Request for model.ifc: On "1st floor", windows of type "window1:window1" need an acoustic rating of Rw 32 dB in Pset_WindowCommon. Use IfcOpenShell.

First a look at what the model holds.

```python
import ifcopenshell
import ifcopenshell.util.element

model = ifcopenshell.open("model.ifc")
print(model.schema)
storey = next(s for s in model.by_type("IfcBuildingStorey") if s.Name == "1st floor")
windows = [e for e in ifcopenshell.util.element.get_decomposition(storey) if e.is_a("IfcWindow")]
seen = {}
for e in windows:
    element_type = ifcopenshell.util.element.get_type(e)
    key = (element_type.Name if element_type != e and element_type else None, ifcopenshell.util.element.get_pset(e, "Pset_WindowCommon", "AcousticRating"))
    seen[key] = seen.get(key, 0) + 1
for (name, value), count in sorted(seen.items(), key=str):
    print(count, "x", name, "|", value)
```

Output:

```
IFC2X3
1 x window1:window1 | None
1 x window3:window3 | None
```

```python
import ifcopenshell
import ifcopenshell.api.pset
import ifcopenshell.util.element

model = ifcopenshell.open("model.ifc")

storey = next(s for s in model.by_type("IfcBuildingStorey") if s.Name == "1st floor")
windows = [e for e in ifcopenshell.util.element.get_decomposition(storey) if e.is_a("IfcWindow")]

count = 0
for e in windows:
    element_type = ifcopenshell.util.element.get_type(e)
    if element_type in (None, e) or element_type.Name != "window1:window1":
        continue
    # add_pset returns the element's existing set when there is one.
    pset = ifcopenshell.api.pset.add_pset(model, product=e, name="Pset_WindowCommon")
    ifcopenshell.api.pset.edit_pset(model, pset=pset, properties={"AcousticRating": "Rw 32 dB"})
    count += 1

print(count, "windows updated")

model.write("model-out.ifc")
```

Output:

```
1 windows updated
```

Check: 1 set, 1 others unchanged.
